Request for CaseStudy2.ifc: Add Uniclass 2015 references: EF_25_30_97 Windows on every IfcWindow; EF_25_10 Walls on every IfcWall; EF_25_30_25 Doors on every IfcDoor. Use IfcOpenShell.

First a look at what the model holds.

```python
import ifcopenshell

model = ifcopenshell.open("CaseStudy2.ifc")
print(model.schema)
print("classifications:", [c.Name for c in model.by_type("IfcClassification")])
for ifc_class in ("IfcDoor", "IfcRoof", "IfcStair", "IfcWall", "IfcWindow"):
    print(ifc_class, len(model.by_type(ifc_class)))
```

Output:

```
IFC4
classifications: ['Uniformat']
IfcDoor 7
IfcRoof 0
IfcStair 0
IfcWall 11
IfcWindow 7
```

```python
import ifcopenshell
import ifcopenshell.api.classification

model = ifcopenshell.open("CaseStudy2.ifc")

system = ifcopenshell.api.classification.add_classification(model, classification="Uniclass 2015")

codes = {
    "IfcWindow": ("EF_25_30_97", "Windows"),
    "IfcWall": ("EF_25_10", "Walls"),
    "IfcDoor": ("EF_25_30_25", "Doors"),
}
for ifc_class, (code, name) in codes.items():
    products = model.by_type(ifc_class)
    ifcopenshell.api.classification.add_reference(
        model, products=products, classification=system, identification=code, name=name
    )
    print(code, len(products))

model.write("CaseStudy2_updated.ifc")
```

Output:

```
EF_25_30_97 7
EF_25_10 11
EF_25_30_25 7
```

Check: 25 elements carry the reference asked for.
